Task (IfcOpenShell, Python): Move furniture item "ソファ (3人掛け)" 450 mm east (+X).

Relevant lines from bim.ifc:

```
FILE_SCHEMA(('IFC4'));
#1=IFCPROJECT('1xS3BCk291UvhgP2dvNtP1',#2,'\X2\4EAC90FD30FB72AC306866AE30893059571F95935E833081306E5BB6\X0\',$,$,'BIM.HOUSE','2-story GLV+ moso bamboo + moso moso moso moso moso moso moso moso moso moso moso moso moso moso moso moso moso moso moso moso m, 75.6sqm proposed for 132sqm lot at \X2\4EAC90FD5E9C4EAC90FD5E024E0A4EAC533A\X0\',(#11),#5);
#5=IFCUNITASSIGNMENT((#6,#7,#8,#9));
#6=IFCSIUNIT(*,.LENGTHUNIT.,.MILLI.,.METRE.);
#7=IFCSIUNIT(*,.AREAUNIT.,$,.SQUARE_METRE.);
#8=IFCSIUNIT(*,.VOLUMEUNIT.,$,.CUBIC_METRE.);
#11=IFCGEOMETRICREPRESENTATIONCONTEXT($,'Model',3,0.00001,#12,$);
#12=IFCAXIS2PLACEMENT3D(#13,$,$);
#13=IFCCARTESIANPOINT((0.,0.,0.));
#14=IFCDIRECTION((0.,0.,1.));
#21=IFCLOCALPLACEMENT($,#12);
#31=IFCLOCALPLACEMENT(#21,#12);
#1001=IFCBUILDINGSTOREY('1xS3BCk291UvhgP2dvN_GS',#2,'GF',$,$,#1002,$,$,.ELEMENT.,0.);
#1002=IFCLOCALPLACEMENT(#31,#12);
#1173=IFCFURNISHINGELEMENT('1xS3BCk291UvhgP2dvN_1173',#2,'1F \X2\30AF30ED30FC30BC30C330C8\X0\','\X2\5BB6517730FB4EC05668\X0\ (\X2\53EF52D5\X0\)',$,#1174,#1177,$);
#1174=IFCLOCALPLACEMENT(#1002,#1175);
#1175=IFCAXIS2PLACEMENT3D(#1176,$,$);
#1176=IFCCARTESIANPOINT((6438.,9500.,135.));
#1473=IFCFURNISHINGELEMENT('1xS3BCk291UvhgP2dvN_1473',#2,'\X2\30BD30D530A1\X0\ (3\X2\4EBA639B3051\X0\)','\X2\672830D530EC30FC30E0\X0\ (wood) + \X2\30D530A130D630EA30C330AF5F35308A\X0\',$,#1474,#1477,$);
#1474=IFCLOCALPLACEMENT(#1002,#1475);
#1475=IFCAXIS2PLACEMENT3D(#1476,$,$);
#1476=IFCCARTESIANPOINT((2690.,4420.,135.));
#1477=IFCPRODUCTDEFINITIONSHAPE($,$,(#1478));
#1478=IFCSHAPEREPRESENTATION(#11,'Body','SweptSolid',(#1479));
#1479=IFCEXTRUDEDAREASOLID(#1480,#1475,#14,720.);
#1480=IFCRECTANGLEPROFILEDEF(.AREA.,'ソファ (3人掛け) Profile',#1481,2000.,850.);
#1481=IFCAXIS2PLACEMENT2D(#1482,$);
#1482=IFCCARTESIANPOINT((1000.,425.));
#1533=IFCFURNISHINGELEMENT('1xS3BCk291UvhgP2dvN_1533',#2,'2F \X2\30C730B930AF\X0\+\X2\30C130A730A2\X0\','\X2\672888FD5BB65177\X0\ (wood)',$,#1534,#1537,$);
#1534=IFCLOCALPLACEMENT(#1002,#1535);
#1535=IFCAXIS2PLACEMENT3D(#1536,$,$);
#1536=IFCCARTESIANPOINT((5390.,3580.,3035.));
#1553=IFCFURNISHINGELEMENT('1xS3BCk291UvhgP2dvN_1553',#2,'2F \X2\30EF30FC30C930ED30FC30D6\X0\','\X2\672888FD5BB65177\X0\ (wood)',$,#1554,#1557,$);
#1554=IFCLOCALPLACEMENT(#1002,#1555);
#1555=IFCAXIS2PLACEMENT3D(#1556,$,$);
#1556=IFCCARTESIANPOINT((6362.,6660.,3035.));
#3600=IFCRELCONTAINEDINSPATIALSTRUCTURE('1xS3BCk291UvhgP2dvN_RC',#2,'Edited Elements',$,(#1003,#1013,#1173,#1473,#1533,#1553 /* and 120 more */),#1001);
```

```python
import ifcopenshell
import ifcopenshell.api.geometry
import ifcopenshell.util.placement

model = ifcopenshell.open("bim.ifc")

item = model.by_id(1473)
matrix = ifcopenshell.util.placement.get_local_placement(item.ObjectPlacement)
matrix[0, 3] += 450.0
ifcopenshell.api.geometry.edit_object_placement(model, product=item, matrix=matrix, is_si=False)

print(ifcopenshell.util.placement.get_local_placement(item.ObjectPlacement).round(3) + 0.0)

model.write("bim_v2.ifc")
```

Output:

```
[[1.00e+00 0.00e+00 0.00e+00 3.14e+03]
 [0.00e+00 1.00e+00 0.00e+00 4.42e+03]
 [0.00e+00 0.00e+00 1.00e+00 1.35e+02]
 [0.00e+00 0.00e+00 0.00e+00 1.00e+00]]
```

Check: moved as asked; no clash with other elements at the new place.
